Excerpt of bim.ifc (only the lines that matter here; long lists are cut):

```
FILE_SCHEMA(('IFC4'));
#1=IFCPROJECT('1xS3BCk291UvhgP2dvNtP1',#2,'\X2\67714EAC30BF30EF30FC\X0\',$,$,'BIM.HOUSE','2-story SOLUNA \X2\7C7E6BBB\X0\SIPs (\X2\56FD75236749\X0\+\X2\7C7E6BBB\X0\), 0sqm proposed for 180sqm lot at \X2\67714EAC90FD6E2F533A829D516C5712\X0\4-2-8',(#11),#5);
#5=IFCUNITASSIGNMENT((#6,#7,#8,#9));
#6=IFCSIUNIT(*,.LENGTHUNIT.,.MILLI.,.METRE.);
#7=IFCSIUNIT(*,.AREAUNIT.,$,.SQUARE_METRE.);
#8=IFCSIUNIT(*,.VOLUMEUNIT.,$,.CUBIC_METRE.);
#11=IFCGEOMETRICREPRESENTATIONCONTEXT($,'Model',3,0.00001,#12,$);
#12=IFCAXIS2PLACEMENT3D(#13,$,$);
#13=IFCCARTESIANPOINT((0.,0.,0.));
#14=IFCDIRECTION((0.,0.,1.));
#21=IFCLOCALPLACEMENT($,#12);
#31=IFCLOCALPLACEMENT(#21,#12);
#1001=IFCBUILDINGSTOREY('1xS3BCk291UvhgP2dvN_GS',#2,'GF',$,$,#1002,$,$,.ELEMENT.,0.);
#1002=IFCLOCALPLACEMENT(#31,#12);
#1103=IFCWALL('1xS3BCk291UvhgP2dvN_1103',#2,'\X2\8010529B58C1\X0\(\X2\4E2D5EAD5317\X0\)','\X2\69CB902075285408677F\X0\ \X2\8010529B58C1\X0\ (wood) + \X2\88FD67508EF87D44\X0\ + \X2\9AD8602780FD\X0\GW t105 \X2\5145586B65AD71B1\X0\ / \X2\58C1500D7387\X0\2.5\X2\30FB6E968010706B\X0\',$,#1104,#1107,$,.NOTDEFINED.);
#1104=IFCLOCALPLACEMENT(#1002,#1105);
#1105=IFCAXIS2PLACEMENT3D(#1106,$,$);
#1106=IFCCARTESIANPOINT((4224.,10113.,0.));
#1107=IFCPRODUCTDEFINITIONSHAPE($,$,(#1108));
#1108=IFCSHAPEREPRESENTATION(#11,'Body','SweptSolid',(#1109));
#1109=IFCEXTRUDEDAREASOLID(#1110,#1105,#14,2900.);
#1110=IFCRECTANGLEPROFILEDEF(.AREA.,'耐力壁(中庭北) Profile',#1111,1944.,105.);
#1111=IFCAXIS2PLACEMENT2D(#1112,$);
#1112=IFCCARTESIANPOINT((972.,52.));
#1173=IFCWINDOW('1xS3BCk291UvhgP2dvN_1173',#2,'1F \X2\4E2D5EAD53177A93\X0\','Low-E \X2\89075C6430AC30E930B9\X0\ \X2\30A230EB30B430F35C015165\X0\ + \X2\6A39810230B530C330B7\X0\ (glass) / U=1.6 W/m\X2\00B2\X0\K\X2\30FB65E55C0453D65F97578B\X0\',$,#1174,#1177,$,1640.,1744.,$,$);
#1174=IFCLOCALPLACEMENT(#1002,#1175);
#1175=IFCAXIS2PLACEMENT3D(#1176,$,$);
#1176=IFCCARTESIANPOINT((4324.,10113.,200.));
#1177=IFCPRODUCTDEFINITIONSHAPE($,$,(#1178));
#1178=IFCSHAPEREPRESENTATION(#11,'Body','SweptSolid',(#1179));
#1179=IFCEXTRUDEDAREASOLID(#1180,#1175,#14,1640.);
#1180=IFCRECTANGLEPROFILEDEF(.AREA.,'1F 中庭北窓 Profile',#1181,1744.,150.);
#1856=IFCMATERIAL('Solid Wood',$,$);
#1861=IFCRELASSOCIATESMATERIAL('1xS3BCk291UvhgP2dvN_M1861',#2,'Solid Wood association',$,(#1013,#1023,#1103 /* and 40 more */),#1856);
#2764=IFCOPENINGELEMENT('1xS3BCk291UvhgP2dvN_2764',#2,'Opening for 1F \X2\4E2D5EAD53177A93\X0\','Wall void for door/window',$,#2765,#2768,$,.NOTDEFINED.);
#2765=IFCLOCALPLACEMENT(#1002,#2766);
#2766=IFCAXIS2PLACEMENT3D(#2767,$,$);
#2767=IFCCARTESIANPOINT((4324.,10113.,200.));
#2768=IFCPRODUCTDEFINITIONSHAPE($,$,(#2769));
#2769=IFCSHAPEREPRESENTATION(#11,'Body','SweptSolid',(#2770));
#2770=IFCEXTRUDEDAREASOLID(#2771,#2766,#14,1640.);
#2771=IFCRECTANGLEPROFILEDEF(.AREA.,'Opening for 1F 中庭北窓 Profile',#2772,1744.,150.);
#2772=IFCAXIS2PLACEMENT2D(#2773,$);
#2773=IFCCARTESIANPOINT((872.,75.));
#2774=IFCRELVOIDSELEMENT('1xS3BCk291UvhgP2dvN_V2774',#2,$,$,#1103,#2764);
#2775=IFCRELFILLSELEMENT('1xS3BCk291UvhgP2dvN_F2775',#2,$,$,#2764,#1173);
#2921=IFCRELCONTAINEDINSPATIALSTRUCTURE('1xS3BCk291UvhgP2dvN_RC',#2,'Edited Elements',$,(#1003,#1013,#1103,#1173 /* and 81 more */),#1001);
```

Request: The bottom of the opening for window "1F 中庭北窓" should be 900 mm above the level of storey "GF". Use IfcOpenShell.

```python
import numpy as np
import ifcopenshell
import ifcopenshell.api.geometry
import ifcopenshell.geom
import ifcopenshell.util.element
import ifcopenshell.util.placement
import ifcopenshell.util.shape
import ifcopenshell.util.unit

model = ifcopenshell.open("bim.ifc")
unit_scale = ifcopenshell.util.unit.calculate_unit_scale(model)

window = model.by_guid("1xS3BCk291UvhgP2dvN_1173")
opening = window.FillsVoids[0].RelatingOpeningElement
storey = ifcopenshell.util.element.get_container(window, ifc_class="IfcBuildingStorey")
level = ifcopenshell.util.placement.get_local_placement(storey.ObjectPlacement)[2, 3]

# The opening's origin need not be at the sill, so measure its lowest point.
shape = ifcopenshell.geom.create_shape(ifcopenshell.geom.settings(), opening)
bottom = ifcopenshell.util.shape.get_shape_bottom_elevation(shape, shape.geometry) / unit_scale
dz = level + 900.0 - bottom

shift = np.array([0.0, 0.0, dz])
# The window is not placed relative to its opening, so move both.
for product in (opening, window):
    matrix = ifcopenshell.util.placement.get_local_placement(product.ObjectPlacement)
    matrix[:3, 3] += shift
    ifcopenshell.api.geometry.edit_object_placement(model, product=product, matrix=matrix, is_si=False)

print(f"moved by {dz * unit_scale:+.3f} m")

model.write("bim_updated.ifc")
```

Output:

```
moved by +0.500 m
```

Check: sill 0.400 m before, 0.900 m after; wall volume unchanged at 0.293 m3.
